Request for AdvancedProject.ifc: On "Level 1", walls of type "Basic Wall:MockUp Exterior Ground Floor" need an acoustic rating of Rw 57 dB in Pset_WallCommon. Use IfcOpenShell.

First a look at what the model holds.

```python
import ifcopenshell
import ifcopenshell.util.element

model = ifcopenshell.open("AdvancedProject.ifc")
print(model.schema)
storey = next(s for s in model.by_type("IfcBuildingStorey") if s.Name == "Level 1")
walls = [e for e in ifcopenshell.util.element.get_decomposition(storey) if e.is_a("IfcWall")]
seen = {}
for e in walls:
    element_type = ifcopenshell.util.element.get_type(e)
    key = (element_type.Name if element_type != e and element_type else None, ifcopenshell.util.element.get_pset(e, "Pset_WallCommon", "AcousticRating"))
    seen[key] = seen.get(key, 0) + 1
for (name, value), count in sorted(seen.items(), key=str):
    print(count, "x", name, "|", value)
```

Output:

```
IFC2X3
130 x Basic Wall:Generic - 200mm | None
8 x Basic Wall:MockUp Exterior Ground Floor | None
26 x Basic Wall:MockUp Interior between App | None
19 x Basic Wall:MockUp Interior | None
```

```python
import ifcopenshell
import ifcopenshell.api.pset
import ifcopenshell.util.element

model = ifcopenshell.open("AdvancedProject.ifc")

storey = next(s for s in model.by_type("IfcBuildingStorey") if s.Name == "Level 1")
walls = [e for e in ifcopenshell.util.element.get_decomposition(storey) if e.is_a("IfcWall")]

count = 0
for e in walls:
    element_type = ifcopenshell.util.element.get_type(e)
    if element_type in (None, e) or element_type.Name != "Basic Wall:MockUp Exterior Ground Floor":
        continue
    # add_pset returns the element's existing set when there is one.
    pset = ifcopenshell.api.pset.add_pset(model, product=e, name="Pset_WallCommon")
    ifcopenshell.api.pset.edit_pset(model, pset=pset, properties={"AcousticRating": "Rw 57 dB"})
    count += 1

print(count, "walls updated")

model.write("AdvancedProject_rev.ifc")
```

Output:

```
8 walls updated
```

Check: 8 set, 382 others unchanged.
